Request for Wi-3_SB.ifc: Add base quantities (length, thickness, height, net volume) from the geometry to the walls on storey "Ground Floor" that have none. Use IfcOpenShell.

First a look at what the model holds.

```python
import ifcopenshell
import ifcopenshell.util.element
import ifcopenshell.util.unit

model = ifcopenshell.open("Wi-3_SB.ifc")
print(model.schema)
for unit_type in ("LENGTHUNIT", "AREAUNIT", "VOLUMEUNIT"):
    print(unit_type, ifcopenshell.util.unit.calculate_unit_scale(model, unit_type))
storey = next(s for s in model.by_type("IfcBuildingStorey") if s.Name == "Ground Floor")
walls = [e for e in ifcopenshell.util.element.get_decomposition(storey) if e.is_a("IfcWall")]
for e in sorted(walls, key=lambda e: e.id()):
    print(e.id(), e.is_a(), e.Name, list(ifcopenshell.util.element.get_psets(e, qtos_only=True)), sep=" | ")
```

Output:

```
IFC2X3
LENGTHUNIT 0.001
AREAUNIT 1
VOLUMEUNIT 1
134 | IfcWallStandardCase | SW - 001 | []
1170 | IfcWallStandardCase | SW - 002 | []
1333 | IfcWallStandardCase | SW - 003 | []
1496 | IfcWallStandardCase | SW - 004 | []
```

```python
import ifcopenshell
import ifcopenshell.api.pset
import ifcopenshell.geom
import ifcopenshell.util.element
import ifcopenshell.util.shape
import ifcopenshell.util.unit

model = ifcopenshell.open("Wi-3_SB.ifc")
unit_scale = ifcopenshell.util.unit.calculate_unit_scale(model)
volume_scale = ifcopenshell.util.unit.calculate_unit_scale(model, "VOLUMEUNIT")
settings = ifcopenshell.geom.settings()

storey = next(s for s in model.by_type("IfcBuildingStorey") if s.Name == "Ground Floor")
walls = [e for e in ifcopenshell.util.element.get_decomposition(storey) if e.is_a("IfcWall")]

for e in sorted(walls, key=lambda e: e.id()):
    if ifcopenshell.util.element.get_psets(e, qtos_only=True, should_inherit=False):
        continue
    # Geometry comes back in metres, in the element's own axes.
    shape = ifcopenshell.geom.create_shape(settings, e)
    values = {
        "Length": ifcopenshell.util.shape.get_x(shape.geometry) / unit_scale,
        "Width": ifcopenshell.util.shape.get_y(shape.geometry) / unit_scale,
        "Height": ifcopenshell.util.shape.get_z(shape.geometry) / unit_scale,
        "NetVolume": ifcopenshell.util.shape.get_volume(shape.geometry) / volume_scale,
    }
    qto = ifcopenshell.api.pset.add_qto(model, product=e, name="BaseQuantities")
    ifcopenshell.api.pset.edit_qto(model, qto=qto, properties=values)
    print(e.id(), {k: round(v, 3) for k, v in values.items()})

model.write("Wi-3_SB_edited.ifc")
```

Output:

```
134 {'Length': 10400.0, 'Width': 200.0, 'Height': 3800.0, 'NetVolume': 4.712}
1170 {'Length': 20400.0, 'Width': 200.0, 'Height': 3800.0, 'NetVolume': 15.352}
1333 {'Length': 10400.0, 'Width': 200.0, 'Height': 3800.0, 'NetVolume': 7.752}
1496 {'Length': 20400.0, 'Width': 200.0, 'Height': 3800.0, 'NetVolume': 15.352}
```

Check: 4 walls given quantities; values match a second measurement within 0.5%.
